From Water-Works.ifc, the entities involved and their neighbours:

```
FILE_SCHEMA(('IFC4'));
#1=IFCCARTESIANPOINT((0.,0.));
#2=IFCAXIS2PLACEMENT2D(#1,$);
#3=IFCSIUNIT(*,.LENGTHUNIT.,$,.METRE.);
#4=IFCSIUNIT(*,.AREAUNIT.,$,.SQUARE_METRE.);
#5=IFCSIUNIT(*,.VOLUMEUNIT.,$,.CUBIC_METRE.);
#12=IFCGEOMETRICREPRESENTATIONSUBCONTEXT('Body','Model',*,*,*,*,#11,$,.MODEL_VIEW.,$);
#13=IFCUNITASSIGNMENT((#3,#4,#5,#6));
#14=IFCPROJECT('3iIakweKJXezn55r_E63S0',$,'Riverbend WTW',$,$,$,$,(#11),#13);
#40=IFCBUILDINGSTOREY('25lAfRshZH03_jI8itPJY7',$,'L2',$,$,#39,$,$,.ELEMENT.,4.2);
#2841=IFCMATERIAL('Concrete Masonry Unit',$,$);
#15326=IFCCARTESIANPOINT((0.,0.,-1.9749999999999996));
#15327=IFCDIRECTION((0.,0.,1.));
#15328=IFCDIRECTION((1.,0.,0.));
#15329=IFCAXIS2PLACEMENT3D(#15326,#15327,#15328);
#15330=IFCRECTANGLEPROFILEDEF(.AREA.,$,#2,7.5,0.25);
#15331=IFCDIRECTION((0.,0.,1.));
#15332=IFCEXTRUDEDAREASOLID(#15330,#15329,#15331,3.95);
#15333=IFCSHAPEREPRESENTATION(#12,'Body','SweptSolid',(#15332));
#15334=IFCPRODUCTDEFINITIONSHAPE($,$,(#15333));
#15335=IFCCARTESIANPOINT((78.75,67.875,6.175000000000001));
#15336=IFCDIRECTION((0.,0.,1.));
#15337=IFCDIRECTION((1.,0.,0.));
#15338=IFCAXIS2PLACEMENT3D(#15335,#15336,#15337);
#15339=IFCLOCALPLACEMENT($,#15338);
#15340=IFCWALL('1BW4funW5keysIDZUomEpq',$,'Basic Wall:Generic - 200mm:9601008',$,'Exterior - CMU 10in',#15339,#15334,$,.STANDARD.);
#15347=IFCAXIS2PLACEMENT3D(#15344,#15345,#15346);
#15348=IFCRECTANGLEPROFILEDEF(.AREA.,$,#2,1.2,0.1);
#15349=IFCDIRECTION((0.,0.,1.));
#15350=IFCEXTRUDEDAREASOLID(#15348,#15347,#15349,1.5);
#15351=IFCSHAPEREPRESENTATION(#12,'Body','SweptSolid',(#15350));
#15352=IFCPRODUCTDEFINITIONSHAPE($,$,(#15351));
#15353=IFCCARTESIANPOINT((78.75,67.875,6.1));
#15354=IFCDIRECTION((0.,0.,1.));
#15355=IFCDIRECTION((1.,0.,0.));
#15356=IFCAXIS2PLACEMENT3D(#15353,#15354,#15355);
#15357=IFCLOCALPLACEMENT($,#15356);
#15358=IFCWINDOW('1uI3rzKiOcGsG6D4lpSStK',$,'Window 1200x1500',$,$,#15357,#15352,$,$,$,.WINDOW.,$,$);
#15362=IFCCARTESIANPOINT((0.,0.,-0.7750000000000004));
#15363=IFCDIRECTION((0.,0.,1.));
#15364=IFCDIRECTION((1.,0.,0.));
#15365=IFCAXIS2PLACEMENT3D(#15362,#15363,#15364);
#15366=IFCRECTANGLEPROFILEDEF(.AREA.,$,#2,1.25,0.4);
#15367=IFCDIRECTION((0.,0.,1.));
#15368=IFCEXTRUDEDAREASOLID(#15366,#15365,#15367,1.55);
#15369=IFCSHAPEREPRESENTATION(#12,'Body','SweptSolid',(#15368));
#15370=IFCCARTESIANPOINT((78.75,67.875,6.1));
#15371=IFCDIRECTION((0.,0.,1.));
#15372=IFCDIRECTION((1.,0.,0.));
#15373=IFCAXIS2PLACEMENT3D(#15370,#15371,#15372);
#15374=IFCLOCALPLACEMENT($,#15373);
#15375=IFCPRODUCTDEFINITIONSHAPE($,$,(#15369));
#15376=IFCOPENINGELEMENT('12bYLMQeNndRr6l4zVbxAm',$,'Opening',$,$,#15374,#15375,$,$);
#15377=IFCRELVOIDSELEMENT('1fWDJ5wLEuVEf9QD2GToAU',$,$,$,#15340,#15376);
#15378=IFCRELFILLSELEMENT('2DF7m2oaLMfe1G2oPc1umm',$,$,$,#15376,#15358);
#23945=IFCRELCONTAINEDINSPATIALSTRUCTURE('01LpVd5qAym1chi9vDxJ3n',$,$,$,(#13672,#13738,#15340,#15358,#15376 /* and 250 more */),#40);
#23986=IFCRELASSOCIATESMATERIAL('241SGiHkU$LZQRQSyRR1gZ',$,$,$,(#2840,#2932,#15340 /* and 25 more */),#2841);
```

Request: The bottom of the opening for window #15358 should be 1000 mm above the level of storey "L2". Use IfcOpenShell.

```python
import numpy as np
import ifcopenshell
import ifcopenshell.api.geometry
import ifcopenshell.geom
import ifcopenshell.util.element
import ifcopenshell.util.placement
import ifcopenshell.util.shape
import ifcopenshell.util.unit

model = ifcopenshell.open("Water-Works.ifc")
unit_scale = ifcopenshell.util.unit.calculate_unit_scale(model)

window = model.by_guid("1uI3rzKiOcGsG6D4lpSStK")
opening = window.FillsVoids[0].RelatingOpeningElement
storey = ifcopenshell.util.element.get_container(window, ifc_class="IfcBuildingStorey")
level = ifcopenshell.util.placement.get_local_placement(storey.ObjectPlacement)[2, 3]

# The opening's origin need not be at the sill, so measure its lowest point.
shape = ifcopenshell.geom.create_shape(ifcopenshell.geom.settings(), opening)
bottom = ifcopenshell.util.shape.get_shape_bottom_elevation(shape, shape.geometry) / unit_scale
dz = level + 1 / unit_scale - bottom

shift = np.array([0.0, 0.0, dz])
# The window is not placed relative to its opening, so move both.
for product in (opening, window):
    matrix = ifcopenshell.util.placement.get_local_placement(product.ObjectPlacement)
    matrix[:3, 3] += shift
    ifcopenshell.api.geometry.edit_object_placement(model, product=product, matrix=matrix, is_si=False)

print(f"moved by {dz * unit_scale:+.3f} m")

model.write("Water-Works_rev.ifc")
```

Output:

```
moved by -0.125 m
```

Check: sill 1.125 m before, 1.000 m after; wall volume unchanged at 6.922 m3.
